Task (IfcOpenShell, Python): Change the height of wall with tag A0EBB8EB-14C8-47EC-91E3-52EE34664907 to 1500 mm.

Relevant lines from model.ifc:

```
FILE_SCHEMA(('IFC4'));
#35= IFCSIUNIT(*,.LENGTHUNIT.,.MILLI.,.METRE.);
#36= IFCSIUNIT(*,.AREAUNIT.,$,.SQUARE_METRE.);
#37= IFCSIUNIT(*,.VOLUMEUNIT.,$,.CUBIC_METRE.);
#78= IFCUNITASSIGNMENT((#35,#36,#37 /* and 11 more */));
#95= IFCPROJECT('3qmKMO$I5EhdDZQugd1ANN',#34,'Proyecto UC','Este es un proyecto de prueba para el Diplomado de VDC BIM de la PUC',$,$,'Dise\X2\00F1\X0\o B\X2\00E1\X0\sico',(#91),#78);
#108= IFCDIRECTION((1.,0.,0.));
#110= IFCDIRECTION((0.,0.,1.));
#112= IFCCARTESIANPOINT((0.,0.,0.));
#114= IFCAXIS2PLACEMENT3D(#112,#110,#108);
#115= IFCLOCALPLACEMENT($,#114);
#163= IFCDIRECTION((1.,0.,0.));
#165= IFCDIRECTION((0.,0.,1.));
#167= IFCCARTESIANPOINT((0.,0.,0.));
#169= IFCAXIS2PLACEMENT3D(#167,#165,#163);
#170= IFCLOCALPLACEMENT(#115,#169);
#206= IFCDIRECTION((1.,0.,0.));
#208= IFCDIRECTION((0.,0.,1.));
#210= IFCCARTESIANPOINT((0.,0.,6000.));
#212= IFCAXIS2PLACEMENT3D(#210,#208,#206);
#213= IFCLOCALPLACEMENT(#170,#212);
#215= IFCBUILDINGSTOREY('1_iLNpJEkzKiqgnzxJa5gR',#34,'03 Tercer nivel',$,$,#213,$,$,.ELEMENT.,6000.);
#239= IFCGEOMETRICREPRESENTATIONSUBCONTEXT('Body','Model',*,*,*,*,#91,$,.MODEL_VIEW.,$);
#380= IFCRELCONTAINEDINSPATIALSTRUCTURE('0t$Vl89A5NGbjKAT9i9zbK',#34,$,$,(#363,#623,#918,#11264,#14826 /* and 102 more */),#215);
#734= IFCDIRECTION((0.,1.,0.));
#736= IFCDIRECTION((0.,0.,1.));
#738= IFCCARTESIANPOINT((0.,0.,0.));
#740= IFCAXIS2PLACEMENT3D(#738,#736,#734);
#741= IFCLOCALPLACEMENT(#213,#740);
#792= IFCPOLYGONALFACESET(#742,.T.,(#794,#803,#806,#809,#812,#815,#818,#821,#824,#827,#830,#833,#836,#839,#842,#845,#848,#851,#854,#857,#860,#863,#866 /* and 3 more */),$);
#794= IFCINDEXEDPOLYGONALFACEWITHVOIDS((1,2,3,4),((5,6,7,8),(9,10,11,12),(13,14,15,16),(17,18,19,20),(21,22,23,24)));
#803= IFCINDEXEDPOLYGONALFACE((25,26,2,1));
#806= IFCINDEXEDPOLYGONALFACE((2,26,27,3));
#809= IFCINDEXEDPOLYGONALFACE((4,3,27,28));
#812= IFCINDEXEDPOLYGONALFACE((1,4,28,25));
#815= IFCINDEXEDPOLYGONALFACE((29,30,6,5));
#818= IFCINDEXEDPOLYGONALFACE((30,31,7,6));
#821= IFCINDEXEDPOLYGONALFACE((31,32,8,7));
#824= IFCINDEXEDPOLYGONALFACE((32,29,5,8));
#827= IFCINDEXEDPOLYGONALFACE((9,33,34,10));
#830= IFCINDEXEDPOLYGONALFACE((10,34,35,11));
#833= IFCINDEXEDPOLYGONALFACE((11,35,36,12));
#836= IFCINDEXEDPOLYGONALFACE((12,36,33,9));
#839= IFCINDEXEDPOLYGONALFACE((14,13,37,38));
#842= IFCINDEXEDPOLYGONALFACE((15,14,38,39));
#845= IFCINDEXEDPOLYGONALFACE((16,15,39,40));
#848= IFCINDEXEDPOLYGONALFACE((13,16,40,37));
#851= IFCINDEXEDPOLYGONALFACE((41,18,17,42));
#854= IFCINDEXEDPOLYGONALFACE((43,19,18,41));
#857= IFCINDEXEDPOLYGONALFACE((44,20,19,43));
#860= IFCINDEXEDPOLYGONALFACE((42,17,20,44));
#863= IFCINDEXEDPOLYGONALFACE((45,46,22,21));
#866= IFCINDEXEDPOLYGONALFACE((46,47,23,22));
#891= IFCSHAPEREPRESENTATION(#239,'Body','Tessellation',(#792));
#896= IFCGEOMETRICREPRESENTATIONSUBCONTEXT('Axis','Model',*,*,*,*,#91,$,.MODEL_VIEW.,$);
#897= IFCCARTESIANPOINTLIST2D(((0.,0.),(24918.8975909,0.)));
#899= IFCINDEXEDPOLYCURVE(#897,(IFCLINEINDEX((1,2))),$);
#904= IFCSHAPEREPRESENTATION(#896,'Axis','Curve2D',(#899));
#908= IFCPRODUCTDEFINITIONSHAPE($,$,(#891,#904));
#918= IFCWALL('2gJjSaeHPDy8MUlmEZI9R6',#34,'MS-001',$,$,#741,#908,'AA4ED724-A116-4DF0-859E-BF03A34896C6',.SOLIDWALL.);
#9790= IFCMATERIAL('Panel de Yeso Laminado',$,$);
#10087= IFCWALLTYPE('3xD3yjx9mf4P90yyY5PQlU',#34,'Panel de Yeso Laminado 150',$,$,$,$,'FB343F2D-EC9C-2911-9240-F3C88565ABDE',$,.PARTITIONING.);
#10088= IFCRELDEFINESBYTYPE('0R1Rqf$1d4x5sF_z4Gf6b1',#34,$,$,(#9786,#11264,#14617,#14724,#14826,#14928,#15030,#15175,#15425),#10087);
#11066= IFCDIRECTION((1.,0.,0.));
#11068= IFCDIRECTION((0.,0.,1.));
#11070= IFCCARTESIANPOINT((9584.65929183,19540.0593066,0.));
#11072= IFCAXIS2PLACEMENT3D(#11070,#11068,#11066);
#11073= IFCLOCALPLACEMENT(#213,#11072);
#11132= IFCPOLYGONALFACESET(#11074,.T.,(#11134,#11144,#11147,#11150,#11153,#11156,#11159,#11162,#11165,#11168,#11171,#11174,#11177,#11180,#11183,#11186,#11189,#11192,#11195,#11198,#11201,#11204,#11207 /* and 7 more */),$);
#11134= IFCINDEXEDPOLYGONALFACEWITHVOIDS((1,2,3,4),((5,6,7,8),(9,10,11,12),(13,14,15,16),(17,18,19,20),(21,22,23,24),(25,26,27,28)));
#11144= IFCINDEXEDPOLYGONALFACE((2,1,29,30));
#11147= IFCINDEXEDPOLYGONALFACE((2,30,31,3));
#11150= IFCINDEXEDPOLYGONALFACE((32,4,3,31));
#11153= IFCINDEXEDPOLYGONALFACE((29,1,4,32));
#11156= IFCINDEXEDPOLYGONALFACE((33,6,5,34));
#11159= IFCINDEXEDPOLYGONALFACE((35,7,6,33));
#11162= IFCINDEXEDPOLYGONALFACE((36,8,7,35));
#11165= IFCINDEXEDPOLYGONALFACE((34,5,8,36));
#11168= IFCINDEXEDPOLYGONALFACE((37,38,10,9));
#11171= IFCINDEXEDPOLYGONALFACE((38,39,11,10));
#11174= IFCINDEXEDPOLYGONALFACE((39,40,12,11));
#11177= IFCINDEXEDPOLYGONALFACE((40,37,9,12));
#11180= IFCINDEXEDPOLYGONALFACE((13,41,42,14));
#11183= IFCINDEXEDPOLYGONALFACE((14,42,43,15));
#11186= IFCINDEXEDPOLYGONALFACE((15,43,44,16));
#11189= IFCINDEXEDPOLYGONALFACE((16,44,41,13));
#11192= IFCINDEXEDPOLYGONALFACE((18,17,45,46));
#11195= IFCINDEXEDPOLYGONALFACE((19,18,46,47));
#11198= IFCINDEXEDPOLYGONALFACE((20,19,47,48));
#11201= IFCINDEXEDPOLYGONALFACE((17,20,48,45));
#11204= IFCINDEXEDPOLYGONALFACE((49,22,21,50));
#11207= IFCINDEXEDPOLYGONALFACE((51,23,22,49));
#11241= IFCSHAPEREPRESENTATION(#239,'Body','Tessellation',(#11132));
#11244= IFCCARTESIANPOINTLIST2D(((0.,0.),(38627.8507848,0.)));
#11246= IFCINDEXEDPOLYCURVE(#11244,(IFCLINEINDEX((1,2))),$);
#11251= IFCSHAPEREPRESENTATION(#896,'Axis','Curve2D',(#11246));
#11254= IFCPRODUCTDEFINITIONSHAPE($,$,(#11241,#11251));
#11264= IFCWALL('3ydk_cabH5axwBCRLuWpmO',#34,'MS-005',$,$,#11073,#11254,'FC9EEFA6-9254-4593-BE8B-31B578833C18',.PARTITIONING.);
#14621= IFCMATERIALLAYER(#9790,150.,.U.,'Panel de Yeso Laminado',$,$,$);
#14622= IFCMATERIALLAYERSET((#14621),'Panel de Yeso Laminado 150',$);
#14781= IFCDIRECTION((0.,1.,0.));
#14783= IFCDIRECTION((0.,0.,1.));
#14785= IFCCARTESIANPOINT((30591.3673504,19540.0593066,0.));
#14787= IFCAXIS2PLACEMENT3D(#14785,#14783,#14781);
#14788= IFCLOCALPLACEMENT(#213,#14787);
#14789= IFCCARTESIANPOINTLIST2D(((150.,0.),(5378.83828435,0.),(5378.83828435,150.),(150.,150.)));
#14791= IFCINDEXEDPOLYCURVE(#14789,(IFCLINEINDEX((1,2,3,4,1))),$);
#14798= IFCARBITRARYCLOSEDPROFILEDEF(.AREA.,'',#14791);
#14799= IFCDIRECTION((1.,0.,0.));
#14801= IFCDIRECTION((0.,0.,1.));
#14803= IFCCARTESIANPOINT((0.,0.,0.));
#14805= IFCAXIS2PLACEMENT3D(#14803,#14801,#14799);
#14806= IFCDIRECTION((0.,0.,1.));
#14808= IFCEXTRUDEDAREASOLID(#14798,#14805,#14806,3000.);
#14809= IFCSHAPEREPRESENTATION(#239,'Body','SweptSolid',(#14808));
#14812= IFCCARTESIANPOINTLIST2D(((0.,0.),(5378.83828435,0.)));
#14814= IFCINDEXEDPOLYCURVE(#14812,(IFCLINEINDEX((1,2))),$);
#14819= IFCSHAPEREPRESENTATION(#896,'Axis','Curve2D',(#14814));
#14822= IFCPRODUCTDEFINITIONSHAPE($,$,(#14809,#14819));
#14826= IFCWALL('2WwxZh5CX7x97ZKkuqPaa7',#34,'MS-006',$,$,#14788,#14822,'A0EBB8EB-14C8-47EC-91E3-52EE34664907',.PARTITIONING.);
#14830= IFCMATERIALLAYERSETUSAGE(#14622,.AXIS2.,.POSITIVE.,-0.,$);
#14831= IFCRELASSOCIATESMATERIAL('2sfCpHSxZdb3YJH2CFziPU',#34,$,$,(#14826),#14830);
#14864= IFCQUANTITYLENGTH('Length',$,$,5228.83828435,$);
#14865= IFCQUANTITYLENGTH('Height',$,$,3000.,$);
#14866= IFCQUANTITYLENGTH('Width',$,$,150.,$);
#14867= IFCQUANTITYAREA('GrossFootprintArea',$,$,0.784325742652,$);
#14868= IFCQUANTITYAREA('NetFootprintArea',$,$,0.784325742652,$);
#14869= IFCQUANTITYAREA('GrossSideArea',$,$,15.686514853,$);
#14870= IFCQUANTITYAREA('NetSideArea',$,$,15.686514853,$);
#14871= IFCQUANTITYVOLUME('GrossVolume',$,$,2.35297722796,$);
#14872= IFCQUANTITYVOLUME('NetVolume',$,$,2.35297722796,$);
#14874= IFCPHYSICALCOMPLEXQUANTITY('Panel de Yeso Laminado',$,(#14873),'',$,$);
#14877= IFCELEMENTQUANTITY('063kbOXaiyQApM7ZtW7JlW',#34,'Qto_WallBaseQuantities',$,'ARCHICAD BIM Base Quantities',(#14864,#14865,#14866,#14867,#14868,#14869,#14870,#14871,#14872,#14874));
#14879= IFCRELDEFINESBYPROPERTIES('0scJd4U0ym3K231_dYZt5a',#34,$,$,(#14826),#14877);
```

```python
import ifcopenshell
import ifcopenshell.api.pset
import ifcopenshell.geom
import ifcopenshell.util.element
import ifcopenshell.util.representation
import ifcopenshell.util.shape
import ifcopenshell.util.unit

model = ifcopenshell.open("model.ifc")
unit_scale = ifcopenshell.util.unit.calculate_unit_scale(model)
area_scale = ifcopenshell.util.unit.calculate_unit_scale(model, "AREAUNIT")
volume_scale = ifcopenshell.util.unit.calculate_unit_scale(model, "VOLUMEUNIT")
settings = ifcopenshell.geom.settings()


def volume(element):
    """Net volume in cubic metres, openings subtracted."""
    shape = ifcopenshell.geom.create_shape(settings, element)
    return ifcopenshell.util.shape.get_volume(shape.geometry)


wall = model.by_id(14826)
before = volume(wall)

body = ifcopenshell.util.representation.get_representation(wall, "Model", "Body")
solid = body.Items[0]
old_height = solid.Depth
solid.Depth = 1.5 / unit_scale
after = volume(wall)
thickness = 0.15  # wall thickness in metres

# Update the stored height, areas and volumes.
qto = model.by_id(ifcopenshell.util.element.get_pset(wall, "Qto_WallBaseQuantities", should_inherit=False)["id"])
ifcopenshell.api.pset.edit_qto(model, qto=qto, properties={
    "Height": solid.Depth,
    "GrossSideArea": ifcopenshell.util.element.get_pset(wall, "Qto_WallBaseQuantities", "GrossSideArea") * solid.Depth / old_height,
    "NetSideArea": after / thickness / area_scale,
    "GrossVolume": ifcopenshell.util.element.get_pset(wall, "Qto_WallBaseQuantities", "GrossVolume") * solid.Depth / old_height,
    "NetVolume": after / volume_scale,
})

print(f"height {old_height:g} -> {solid.Depth:g}, volume {before:.3f} -> {after:.3f} m3")

model.write("model-out.ifc")
```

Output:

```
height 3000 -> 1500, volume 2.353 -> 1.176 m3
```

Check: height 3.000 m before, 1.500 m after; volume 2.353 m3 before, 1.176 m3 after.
